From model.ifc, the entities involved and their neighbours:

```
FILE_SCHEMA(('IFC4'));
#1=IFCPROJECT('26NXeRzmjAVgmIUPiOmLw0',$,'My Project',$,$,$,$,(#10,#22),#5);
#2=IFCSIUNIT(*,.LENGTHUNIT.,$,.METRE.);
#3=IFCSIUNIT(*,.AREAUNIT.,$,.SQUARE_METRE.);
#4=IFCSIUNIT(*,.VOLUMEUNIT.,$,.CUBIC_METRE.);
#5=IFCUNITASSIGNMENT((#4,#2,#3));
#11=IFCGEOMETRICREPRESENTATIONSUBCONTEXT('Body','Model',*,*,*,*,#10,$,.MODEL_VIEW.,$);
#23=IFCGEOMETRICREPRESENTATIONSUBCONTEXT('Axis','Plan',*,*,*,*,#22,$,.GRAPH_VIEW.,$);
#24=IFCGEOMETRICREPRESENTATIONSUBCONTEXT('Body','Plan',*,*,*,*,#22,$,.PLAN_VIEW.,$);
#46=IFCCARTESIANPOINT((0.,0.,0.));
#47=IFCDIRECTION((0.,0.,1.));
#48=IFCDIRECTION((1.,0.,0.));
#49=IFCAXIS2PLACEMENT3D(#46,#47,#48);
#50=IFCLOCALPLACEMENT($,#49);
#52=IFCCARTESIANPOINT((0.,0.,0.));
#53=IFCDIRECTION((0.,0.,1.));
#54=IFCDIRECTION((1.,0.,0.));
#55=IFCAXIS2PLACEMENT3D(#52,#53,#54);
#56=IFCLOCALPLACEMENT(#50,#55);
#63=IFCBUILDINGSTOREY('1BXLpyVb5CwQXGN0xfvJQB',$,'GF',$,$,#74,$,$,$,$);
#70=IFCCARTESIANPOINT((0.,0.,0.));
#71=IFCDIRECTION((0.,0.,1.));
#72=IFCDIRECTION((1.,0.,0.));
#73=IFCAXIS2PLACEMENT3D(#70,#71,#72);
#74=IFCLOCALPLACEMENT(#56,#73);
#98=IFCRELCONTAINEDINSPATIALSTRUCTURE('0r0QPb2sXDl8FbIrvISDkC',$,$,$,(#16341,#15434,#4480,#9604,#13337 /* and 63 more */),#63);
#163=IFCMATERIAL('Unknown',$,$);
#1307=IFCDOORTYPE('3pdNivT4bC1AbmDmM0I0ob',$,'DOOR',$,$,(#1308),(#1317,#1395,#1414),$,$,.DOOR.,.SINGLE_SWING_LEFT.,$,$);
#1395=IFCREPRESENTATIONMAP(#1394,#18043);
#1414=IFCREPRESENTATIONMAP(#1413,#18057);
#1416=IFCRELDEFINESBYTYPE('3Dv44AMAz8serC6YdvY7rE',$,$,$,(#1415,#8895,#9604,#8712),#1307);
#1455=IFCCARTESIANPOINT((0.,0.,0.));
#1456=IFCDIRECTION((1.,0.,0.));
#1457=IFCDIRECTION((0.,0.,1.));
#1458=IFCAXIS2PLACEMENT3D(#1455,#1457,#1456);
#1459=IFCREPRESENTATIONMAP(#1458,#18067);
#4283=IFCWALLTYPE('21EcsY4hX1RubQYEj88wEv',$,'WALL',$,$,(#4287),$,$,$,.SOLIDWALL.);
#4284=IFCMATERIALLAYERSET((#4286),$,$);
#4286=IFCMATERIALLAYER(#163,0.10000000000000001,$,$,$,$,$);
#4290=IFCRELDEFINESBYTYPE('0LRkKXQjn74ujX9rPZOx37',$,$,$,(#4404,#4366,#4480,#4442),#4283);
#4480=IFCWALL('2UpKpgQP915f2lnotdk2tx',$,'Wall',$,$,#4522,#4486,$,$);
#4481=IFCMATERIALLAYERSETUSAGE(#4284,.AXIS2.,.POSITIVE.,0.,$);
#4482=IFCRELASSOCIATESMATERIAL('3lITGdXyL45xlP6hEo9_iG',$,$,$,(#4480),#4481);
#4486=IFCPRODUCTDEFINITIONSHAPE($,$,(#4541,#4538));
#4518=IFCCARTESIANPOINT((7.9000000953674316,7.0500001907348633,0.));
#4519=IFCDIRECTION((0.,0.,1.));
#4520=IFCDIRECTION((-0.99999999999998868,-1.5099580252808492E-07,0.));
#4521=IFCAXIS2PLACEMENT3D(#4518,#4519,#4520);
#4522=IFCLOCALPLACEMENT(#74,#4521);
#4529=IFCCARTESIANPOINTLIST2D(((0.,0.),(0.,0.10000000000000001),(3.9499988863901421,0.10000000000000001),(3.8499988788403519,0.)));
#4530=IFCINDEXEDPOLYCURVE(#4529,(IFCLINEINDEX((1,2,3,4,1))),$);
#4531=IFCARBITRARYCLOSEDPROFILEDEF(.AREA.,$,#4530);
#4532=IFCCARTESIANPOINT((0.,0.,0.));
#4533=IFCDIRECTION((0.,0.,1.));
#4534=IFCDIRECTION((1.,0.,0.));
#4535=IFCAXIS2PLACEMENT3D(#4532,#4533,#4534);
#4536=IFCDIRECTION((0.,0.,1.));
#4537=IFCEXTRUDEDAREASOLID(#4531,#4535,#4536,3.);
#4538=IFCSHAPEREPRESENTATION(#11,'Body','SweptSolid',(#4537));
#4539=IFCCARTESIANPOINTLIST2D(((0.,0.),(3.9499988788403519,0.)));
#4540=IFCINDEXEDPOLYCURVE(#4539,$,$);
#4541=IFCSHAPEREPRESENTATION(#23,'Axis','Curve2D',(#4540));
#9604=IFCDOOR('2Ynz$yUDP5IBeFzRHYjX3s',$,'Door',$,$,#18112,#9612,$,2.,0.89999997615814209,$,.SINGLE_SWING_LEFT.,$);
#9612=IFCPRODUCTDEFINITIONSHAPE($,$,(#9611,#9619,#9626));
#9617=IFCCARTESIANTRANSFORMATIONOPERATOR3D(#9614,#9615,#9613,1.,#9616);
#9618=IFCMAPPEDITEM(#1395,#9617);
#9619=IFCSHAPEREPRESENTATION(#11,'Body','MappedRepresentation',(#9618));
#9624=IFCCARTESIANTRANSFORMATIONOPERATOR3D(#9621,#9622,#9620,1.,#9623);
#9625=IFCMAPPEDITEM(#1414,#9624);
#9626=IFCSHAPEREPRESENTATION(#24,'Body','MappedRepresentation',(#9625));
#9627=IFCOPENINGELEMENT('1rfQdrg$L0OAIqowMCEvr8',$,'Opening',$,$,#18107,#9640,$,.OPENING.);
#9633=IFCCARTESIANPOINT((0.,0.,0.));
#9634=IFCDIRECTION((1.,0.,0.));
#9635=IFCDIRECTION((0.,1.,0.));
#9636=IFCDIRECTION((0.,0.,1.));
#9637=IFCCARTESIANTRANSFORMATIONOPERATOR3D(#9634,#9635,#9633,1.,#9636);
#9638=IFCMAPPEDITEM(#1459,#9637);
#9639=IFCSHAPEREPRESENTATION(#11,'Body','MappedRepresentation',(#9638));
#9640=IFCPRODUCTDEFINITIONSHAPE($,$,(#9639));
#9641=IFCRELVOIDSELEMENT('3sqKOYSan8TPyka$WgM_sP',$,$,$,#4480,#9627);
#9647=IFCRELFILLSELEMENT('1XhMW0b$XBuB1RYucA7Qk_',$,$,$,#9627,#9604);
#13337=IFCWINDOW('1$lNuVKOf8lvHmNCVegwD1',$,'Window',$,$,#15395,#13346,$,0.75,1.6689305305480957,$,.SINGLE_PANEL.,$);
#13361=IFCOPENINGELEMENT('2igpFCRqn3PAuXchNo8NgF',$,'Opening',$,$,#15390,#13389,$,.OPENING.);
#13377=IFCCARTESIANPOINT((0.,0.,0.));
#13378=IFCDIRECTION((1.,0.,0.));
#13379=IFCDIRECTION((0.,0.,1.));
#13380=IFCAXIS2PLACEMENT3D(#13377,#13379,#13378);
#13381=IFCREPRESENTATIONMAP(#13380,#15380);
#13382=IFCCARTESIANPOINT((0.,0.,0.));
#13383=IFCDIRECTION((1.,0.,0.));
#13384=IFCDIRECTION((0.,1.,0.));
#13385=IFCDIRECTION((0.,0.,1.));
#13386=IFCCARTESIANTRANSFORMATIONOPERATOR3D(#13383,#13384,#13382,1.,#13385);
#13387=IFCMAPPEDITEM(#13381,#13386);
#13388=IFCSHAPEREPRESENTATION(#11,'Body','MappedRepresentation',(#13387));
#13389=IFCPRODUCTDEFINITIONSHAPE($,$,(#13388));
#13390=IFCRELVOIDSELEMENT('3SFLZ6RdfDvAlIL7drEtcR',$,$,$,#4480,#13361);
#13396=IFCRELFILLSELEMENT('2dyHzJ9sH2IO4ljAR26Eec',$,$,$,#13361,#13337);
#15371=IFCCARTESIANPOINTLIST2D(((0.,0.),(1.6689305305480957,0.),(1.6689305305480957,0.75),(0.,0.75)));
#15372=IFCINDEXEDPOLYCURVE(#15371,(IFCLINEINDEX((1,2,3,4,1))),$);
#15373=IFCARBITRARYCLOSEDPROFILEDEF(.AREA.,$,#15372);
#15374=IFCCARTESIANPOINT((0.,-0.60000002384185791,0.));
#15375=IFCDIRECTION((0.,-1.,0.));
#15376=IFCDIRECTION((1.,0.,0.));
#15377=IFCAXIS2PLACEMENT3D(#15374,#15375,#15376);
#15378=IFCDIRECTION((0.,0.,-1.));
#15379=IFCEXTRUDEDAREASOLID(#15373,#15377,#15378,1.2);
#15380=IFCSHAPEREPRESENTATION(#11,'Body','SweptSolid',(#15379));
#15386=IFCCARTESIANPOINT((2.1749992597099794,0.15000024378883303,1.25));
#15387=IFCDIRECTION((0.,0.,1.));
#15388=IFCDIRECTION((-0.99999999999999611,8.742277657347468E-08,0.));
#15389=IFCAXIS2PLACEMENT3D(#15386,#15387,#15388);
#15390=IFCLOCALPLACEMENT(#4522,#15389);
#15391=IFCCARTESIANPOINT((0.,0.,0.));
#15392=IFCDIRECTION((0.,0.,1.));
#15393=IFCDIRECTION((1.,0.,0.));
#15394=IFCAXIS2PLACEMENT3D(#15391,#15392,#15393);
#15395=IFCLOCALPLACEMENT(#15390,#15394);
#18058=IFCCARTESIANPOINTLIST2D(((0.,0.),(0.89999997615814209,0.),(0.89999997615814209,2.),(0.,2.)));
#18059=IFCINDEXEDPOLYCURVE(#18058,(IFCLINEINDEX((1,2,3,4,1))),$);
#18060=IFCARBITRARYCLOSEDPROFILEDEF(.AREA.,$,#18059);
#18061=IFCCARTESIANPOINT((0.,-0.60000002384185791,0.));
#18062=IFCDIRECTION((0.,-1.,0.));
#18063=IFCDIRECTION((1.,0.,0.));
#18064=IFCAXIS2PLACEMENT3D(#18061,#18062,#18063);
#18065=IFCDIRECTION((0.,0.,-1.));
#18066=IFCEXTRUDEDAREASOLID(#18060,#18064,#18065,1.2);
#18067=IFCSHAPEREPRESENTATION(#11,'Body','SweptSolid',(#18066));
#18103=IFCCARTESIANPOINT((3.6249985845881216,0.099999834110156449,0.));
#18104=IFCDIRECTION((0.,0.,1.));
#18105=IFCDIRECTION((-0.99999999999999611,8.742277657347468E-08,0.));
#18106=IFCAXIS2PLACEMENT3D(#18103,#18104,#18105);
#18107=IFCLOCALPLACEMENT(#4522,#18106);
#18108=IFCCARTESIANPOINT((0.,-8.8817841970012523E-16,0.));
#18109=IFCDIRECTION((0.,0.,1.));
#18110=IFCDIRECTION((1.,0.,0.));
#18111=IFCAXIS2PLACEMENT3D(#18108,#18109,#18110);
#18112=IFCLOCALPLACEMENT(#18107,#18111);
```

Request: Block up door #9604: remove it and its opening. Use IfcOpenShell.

```python
import ifcopenshell
import ifcopenshell.api.feature
import ifcopenshell.api.root
import ifcopenshell.geom
import ifcopenshell.util.shape

model = ifcopenshell.open("model.ifc")
settings = ifcopenshell.geom.settings()


def volume(element):
    """Net volume in cubic metres, openings subtracted."""
    shape = ifcopenshell.geom.create_shape(settings, element)
    return ifcopenshell.util.shape.get_volume(shape.geometry)


door = model.by_guid("2Ynz$yUDP5IBeFzRHYjX3s")
opening = door.FillsVoids[0].RelatingOpeningElement
wall = opening.VoidsElements[0].RelatingBuildingElement
before = volume(wall)

ifcopenshell.api.root.remove_product(model, product=door)
ifcopenshell.api.feature.remove_feature(model, feature=opening)

after = volume(wall)

print(f"wall volume {before:.3f} -> {after:.3f} m3")

model.write("model_edited.ifc")
```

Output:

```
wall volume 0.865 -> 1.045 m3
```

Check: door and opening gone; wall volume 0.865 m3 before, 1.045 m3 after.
